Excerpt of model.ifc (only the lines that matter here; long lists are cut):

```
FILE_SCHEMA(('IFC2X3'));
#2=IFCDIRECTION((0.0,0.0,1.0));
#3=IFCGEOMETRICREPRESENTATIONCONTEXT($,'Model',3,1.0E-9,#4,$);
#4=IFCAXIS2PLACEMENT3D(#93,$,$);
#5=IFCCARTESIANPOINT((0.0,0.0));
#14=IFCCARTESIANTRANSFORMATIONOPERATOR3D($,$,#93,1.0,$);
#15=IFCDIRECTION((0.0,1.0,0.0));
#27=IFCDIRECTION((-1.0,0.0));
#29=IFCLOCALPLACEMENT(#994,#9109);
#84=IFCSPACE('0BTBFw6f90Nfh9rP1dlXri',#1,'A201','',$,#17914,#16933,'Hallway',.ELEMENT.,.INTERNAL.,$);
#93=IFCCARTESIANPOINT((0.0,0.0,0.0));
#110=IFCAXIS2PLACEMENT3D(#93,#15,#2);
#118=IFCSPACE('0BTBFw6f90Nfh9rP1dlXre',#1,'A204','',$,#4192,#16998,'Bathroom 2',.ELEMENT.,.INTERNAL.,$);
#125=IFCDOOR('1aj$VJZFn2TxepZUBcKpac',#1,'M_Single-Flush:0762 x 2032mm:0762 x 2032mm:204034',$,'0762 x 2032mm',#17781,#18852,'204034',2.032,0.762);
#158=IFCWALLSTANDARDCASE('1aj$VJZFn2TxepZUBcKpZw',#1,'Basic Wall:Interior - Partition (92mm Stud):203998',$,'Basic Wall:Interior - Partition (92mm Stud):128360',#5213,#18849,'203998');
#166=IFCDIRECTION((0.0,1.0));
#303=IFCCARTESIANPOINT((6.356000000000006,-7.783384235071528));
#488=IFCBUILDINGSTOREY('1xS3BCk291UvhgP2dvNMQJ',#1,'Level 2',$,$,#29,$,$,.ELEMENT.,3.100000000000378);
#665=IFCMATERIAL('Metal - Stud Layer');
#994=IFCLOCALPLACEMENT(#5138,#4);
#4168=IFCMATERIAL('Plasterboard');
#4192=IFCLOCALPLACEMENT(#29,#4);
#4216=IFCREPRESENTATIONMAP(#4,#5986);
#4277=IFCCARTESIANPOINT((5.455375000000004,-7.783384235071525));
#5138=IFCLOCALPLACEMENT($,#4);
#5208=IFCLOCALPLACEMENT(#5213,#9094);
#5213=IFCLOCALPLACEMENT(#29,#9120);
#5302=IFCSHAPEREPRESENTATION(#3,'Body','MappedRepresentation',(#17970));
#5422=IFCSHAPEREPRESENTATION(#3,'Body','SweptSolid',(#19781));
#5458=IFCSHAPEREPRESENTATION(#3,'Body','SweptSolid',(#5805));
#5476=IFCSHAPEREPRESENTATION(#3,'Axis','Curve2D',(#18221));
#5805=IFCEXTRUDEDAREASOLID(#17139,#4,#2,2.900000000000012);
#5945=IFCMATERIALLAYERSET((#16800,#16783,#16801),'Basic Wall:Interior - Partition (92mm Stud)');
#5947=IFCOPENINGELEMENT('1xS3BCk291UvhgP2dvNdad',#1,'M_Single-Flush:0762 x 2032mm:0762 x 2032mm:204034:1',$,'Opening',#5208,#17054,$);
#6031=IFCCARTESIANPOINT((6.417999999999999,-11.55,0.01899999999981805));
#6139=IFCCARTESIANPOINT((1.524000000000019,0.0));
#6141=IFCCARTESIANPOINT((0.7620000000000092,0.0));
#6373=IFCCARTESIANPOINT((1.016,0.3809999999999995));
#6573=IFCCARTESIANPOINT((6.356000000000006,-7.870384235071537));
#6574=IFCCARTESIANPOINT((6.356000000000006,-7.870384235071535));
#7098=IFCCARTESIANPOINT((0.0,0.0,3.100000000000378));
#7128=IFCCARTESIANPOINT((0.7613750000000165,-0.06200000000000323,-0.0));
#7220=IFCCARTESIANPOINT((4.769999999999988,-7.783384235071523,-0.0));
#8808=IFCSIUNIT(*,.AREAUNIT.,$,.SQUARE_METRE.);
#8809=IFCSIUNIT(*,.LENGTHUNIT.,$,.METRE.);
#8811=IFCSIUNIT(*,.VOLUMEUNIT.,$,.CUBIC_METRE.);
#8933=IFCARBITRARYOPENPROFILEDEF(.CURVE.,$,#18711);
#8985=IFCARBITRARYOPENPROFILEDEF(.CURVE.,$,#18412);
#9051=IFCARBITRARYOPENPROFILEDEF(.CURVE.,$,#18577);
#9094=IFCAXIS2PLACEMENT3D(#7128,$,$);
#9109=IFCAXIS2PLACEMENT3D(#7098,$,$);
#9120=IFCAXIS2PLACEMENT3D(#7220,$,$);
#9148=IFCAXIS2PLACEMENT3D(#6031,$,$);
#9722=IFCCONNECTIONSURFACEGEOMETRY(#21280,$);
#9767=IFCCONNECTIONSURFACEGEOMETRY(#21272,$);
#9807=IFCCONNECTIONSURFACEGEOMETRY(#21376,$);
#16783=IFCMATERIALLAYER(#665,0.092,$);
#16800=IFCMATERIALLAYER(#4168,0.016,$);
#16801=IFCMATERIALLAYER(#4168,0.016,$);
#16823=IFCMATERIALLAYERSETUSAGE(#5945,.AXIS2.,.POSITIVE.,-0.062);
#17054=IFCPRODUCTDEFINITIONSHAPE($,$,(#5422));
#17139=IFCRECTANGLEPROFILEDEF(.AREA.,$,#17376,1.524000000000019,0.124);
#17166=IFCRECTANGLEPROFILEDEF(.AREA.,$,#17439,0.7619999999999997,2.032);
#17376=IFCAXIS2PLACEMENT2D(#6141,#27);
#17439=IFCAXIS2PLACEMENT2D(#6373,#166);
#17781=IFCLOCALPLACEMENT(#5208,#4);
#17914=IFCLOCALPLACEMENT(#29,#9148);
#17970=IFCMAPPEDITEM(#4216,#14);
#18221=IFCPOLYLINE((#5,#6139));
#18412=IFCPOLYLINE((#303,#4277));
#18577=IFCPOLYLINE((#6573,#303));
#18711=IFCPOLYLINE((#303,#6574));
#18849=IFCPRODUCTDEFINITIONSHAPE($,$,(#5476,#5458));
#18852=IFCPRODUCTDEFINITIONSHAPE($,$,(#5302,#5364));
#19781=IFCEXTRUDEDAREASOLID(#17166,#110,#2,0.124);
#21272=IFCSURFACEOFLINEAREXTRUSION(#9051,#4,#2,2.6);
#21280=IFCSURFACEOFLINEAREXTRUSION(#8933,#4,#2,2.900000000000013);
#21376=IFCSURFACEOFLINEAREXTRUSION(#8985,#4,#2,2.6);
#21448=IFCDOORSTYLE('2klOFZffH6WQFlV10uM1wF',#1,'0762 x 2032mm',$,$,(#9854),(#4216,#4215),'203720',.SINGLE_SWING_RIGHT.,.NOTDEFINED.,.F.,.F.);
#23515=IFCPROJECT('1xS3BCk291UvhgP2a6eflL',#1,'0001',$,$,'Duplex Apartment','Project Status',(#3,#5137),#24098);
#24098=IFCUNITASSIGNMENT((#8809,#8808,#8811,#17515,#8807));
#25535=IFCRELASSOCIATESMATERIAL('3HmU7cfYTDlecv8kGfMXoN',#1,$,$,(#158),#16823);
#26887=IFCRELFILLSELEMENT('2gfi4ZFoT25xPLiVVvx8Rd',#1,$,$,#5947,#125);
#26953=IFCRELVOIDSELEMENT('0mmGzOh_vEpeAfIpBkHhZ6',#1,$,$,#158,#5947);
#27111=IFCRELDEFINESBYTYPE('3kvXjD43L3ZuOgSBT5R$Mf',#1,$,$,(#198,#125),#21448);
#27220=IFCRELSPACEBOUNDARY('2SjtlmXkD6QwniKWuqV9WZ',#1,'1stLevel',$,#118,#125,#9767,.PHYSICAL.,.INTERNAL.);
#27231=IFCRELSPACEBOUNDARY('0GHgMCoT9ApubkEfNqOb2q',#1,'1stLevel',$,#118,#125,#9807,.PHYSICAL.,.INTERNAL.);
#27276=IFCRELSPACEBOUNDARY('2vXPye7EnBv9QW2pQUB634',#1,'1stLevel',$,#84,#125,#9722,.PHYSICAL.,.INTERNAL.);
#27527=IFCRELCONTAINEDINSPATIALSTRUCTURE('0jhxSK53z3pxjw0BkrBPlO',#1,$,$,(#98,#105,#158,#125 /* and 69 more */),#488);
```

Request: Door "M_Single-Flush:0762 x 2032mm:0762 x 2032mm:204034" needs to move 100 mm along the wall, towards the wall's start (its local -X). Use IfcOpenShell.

```python
import numpy as np
import ifcopenshell
import ifcopenshell.api.geometry
import ifcopenshell.util.placement
import ifcopenshell.util.unit

model = ifcopenshell.open("model.ifc")
unit_scale = ifcopenshell.util.unit.calculate_unit_scale(model)

door = model.by_guid("1aj$VJZFn2TxepZUBcKpac")
opening = door.FillsVoids[0].RelatingOpeningElement
wall = opening.VoidsElements[0].RelatingBuildingElement

wall_matrix = ifcopenshell.util.placement.get_local_placement(wall.ObjectPlacement)
shift = wall_matrix[:3, 0] * -0.1 / unit_scale
before = ifcopenshell.util.placement.get_local_placement(door.ObjectPlacement)[:3, 3].copy()

# The door is placed relative to its opening, so it follows when the opening moves.
matrix = ifcopenshell.util.placement.get_local_placement(opening.ObjectPlacement)
matrix[:3, 3] += shift
ifcopenshell.api.geometry.edit_object_placement(
    model, product=opening, matrix=matrix, is_si=False, should_transform_children=True
)

# Space boundary surfaces are stored in each space's coordinates; move them too.
for rel in door.ProvidesBoundaries:
    if not rel.ConnectionGeometry:
        continue
    surface = rel.ConnectionGeometry.SurfaceOnRelatingElement
    space_matrix = ifcopenshell.util.placement.get_local_placement(rel.RelatingSpace.ObjectPlacement)
    point = np.array(surface.Position.Location.Coordinates) + space_matrix[:3, :3].T @ shift
    surface.Position = model.createIfcAxis2Placement3D(
        model.createIfcCartesianPoint(point.tolist()), surface.Position.Axis, surface.Position.RefDirection
    )

after = ifcopenshell.util.placement.get_local_placement(door.ObjectPlacement)[:3, 3]
print("door moved by", (after - before).round(3) + 0.0)

model.write("model-out.ifc")
```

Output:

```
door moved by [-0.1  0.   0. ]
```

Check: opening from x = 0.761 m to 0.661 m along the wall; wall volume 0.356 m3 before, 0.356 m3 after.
